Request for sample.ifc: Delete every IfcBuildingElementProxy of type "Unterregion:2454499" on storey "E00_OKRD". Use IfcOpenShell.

First a look at what the model holds.

```python
import ifcopenshell
import ifcopenshell.util.element

model = ifcopenshell.open("sample.ifc")
print(model.schema)
storey = next(s for s in model.by_type("IfcBuildingStorey") if s.Name == "E00_OKRD")
proxies = [e for e in ifcopenshell.util.element.get_decomposition(storey) if e.is_a("IfcBuildingElementProxy")]
seen = {}
for e in proxies:
    element_type = ifcopenshell.util.element.get_type(e)
    name = element_type.Name if element_type not in (None, e) else None
    seen[name] = seen.get(name, 0) + 1
for name, count in sorted(seen.items(), key=str):
    print(count, "x", name)
```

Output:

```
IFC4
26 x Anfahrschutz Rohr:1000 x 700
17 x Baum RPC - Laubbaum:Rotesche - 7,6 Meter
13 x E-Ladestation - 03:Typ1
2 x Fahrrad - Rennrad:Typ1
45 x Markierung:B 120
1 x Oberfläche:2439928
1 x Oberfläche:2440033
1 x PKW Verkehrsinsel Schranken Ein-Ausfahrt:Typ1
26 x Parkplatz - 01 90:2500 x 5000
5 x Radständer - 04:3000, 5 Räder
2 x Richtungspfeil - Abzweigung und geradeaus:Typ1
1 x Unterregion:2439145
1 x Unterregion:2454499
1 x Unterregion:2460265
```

```python
import ifcopenshell
import ifcopenshell.api.root
import ifcopenshell.util.element

model = ifcopenshell.open("sample.ifc")

storey = next(s for s in model.by_type("IfcBuildingStorey") if s.Name == "E00_OKRD")
proxies = [e for e in ifcopenshell.util.element.get_decomposition(storey) if e.is_a("IfcBuildingElementProxy")]
targets = [e for e in proxies if (t := ifcopenshell.util.element.get_type(e)) not in (None, e) and t.Name == "Unterregion:2454499"]

for e in targets:
    ifcopenshell.api.root.remove_product(model, product=e)
print(len(targets), "removed")

model.write("sample_v2.ifc")
```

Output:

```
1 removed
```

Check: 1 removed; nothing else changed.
